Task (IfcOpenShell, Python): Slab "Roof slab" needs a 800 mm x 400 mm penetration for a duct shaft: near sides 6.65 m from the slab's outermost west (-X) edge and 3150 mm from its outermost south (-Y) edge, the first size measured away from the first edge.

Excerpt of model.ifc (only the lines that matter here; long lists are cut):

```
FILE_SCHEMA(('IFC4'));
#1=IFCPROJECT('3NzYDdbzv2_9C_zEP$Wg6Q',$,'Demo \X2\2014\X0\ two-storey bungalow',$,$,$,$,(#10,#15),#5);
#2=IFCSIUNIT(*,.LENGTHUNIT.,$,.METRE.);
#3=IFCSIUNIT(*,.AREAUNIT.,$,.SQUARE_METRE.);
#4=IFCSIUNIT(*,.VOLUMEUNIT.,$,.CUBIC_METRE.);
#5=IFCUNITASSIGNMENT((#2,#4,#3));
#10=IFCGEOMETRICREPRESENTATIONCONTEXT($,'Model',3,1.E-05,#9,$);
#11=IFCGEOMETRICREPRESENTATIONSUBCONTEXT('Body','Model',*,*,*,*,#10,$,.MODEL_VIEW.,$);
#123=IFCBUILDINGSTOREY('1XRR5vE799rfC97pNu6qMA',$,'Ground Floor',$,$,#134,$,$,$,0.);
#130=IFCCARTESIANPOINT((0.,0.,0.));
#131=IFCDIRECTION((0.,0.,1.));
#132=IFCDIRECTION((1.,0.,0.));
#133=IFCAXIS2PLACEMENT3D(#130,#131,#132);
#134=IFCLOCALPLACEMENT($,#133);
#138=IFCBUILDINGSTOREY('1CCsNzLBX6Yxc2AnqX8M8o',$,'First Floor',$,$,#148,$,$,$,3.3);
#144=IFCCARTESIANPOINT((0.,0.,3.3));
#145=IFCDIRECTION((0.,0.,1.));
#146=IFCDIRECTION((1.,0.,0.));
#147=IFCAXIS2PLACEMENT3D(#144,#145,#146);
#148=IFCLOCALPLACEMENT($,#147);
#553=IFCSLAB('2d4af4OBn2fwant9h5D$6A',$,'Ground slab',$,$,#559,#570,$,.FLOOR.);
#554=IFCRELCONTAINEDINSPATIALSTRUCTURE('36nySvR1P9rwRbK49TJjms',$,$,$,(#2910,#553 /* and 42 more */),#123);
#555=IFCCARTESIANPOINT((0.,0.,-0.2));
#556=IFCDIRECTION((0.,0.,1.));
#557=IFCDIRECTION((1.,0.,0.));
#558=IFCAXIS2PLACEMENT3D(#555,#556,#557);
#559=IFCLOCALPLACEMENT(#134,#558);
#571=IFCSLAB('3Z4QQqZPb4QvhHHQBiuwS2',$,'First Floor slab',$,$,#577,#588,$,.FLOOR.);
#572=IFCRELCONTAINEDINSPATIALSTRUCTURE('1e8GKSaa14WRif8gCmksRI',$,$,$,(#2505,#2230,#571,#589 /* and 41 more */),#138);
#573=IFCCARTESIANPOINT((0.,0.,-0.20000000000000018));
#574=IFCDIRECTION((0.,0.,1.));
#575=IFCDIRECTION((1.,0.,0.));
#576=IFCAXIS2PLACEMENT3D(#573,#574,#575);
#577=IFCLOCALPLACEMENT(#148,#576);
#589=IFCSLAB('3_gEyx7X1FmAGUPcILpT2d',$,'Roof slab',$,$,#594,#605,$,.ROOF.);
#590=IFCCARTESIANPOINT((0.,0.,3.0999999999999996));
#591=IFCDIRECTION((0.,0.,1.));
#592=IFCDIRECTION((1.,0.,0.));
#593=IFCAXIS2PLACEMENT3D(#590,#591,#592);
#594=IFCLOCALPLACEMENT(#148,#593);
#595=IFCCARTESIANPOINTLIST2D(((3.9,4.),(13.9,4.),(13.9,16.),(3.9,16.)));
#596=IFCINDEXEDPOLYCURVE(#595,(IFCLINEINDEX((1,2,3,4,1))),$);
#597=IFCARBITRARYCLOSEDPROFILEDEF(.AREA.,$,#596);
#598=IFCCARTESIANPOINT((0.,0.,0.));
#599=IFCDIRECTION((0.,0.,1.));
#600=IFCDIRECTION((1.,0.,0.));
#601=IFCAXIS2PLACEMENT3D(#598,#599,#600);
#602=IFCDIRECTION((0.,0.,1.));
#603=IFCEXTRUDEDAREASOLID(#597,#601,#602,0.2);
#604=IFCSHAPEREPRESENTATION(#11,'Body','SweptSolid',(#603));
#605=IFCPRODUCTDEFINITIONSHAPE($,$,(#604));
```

```python
import numpy as np
import ifcopenshell
import ifcopenshell.api.feature
import ifcopenshell.api.geometry
import ifcopenshell.api.root
import ifcopenshell.geom
import ifcopenshell.util.placement
import ifcopenshell.util.representation
import ifcopenshell.util.shape
import ifcopenshell.util.unit

model = ifcopenshell.open("model.ifc")
unit_scale = ifcopenshell.util.unit.calculate_unit_scale(model)
settings = ifcopenshell.geom.settings()


def volume(element):
    """Net volume in cubic metres, openings subtracted."""
    shape = ifcopenshell.geom.create_shape(settings, element)
    return ifcopenshell.util.shape.get_volume(shape.geometry)


slab = model.by_id(589)
before = volume(slab)

# Extent in the slab's own axes, in metres. The edges named are its -X and -Y sides.
slab_shape = ifcopenshell.geom.create_shape(settings, slab)
vertices = ifcopenshell.util.shape.get_vertices(slab_shape.geometry)
x_min, y_min, bottom = vertices.min(axis=0)
top = vertices[:, 2].max()

opening = ifcopenshell.api.root.create_entity(model, ifc_class="IfcOpeningElement", name="Duct shaft opening", predefined_type="OPENING")
context = ifcopenshell.util.representation.get_context(model, "Model", "Body", "MODEL_VIEW")
width, depth = 0.8, 0.4
outline = [(0.0, 0.0), (width, 0.0), (width, depth), (0.0, depth), (0.0, 0.0)]
# Overshoot both faces by 50 mm so the cut is clean.
shape = ifcopenshell.api.geometry.add_slab_representation(
    model, context=context, depth=top - bottom + 0.1, polyline=outline
)
ifcopenshell.api.geometry.assign_representation(model, product=opening, representation=shape)

matrix = ifcopenshell.util.placement.get_local_placement(slab.ObjectPlacement)
matrix[:, 3] = matrix @ np.append(np.array([x_min + 6.65, y_min + 3.15, bottom - 0.05]) / unit_scale, 1.0)
ifcopenshell.api.geometry.edit_object_placement(model, product=opening, matrix=matrix, is_si=False)
ifcopenshell.api.feature.add_feature(model, feature=opening, element=slab)

after = volume(slab)

print(f"slab volume {before:.3f} -> {after:.3f} m3")

model.write("model_edited.ifc")
```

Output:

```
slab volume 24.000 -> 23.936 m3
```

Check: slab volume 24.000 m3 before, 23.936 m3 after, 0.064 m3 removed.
